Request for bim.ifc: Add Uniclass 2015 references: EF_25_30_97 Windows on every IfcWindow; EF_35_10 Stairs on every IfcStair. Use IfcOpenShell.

First a look at what the model holds.

```python
import ifcopenshell

model = ifcopenshell.open("bim.ifc")
print(model.schema)
print("classifications:", [c.Name for c in model.by_type("IfcClassification")])
for ifc_class in ("IfcDoor", "IfcRoof", "IfcStair", "IfcWall", "IfcWindow"):
    print(ifc_class, len(model.by_type(ifc_class)))
```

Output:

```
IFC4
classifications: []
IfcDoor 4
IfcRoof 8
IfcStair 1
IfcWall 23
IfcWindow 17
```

```python
import ifcopenshell
import ifcopenshell.api.classification

model = ifcopenshell.open("bim.ifc")

system = ifcopenshell.api.classification.add_classification(model, classification="Uniclass 2015")

codes = {
    "IfcWindow": ("EF_25_30_97", "Windows"),
    "IfcStair": ("EF_35_10", "Stairs"),
}
for ifc_class, (code, name) in codes.items():
    products = model.by_type(ifc_class)
    ifcopenshell.api.classification.add_reference(
        model, products=products, classification=system, identification=code, name=name
    )
    print(code, len(products))

model.write("bim_updated.ifc")
```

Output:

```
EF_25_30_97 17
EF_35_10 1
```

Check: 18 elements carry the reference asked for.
